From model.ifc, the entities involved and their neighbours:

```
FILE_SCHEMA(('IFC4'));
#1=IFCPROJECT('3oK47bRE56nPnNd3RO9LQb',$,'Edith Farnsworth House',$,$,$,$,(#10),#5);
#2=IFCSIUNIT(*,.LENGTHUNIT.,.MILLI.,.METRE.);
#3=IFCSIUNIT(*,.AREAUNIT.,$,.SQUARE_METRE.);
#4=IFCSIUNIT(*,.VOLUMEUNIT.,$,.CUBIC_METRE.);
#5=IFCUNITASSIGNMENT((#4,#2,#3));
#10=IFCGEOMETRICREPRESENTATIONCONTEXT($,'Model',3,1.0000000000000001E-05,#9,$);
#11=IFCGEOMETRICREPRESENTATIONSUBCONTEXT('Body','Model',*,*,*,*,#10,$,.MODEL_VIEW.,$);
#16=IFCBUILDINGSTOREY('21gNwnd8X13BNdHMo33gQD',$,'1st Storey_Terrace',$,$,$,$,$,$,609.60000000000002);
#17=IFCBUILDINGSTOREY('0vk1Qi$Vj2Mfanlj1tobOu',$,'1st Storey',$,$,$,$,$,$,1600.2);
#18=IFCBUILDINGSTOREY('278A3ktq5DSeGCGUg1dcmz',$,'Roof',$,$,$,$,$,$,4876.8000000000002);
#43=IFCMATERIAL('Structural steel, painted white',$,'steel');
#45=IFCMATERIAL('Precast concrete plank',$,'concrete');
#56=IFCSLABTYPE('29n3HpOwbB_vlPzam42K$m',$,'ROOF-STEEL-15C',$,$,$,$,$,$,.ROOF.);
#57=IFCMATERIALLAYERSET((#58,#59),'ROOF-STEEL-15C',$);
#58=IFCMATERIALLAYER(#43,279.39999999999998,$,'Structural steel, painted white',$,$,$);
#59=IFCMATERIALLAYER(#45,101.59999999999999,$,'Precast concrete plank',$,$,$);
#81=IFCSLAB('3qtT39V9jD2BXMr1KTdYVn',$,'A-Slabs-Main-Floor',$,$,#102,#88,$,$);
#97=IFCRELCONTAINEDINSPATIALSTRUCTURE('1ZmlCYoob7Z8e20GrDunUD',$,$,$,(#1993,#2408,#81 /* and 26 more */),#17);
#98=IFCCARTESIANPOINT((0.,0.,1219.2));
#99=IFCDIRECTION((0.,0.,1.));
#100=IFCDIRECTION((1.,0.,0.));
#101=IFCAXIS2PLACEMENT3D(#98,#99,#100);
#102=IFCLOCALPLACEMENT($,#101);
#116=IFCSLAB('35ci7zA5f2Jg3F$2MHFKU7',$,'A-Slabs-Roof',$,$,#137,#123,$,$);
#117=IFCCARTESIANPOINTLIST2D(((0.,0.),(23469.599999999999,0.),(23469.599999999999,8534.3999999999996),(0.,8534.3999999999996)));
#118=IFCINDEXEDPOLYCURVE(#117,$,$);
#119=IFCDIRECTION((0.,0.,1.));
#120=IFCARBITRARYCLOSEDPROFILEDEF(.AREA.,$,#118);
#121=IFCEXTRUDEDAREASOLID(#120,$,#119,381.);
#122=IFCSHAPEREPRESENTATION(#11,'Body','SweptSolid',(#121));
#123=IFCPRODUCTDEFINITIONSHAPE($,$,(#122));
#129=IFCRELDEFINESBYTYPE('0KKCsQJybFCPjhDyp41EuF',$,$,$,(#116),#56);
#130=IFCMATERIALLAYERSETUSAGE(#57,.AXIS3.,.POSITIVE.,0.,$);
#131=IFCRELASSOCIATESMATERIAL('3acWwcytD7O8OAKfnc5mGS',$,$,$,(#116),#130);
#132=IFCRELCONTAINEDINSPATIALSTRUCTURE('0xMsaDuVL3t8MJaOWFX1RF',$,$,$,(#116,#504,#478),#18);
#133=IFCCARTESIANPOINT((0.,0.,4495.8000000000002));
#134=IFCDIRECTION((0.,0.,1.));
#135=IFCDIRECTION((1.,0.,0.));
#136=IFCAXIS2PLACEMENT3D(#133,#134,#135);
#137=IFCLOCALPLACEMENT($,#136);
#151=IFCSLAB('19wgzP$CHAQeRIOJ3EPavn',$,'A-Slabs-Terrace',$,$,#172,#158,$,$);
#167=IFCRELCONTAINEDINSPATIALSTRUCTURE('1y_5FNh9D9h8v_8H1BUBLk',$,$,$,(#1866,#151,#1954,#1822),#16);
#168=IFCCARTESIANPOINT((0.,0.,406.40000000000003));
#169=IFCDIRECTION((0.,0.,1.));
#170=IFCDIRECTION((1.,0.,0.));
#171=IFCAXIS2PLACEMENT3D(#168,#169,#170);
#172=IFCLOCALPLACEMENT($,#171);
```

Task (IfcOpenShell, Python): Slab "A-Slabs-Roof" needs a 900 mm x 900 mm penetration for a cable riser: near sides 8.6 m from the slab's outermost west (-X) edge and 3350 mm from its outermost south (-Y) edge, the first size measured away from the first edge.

```python
import numpy as np
import ifcopenshell
import ifcopenshell.api.feature
import ifcopenshell.api.geometry
import ifcopenshell.api.root
import ifcopenshell.geom
import ifcopenshell.util.placement
import ifcopenshell.util.representation
import ifcopenshell.util.shape
import ifcopenshell.util.unit

model = ifcopenshell.open("model.ifc")
unit_scale = ifcopenshell.util.unit.calculate_unit_scale(model)
settings = ifcopenshell.geom.settings()


def volume(element):
    """Net volume in cubic metres, openings subtracted."""
    shape = ifcopenshell.geom.create_shape(settings, element)
    return ifcopenshell.util.shape.get_volume(shape.geometry)


slab = model.by_guid("35ci7zA5f2Jg3F$2MHFKU7")
before = volume(slab)

# Extent in the slab's own axes, in metres. The edges named are its -X and -Y sides.
slab_shape = ifcopenshell.geom.create_shape(settings, slab)
vertices = ifcopenshell.util.shape.get_vertices(slab_shape.geometry)
x_min, y_min, bottom = vertices.min(axis=0)
top = vertices[:, 2].max()

opening = ifcopenshell.api.root.create_entity(model, ifc_class="IfcOpeningElement", name="Cable riser opening", predefined_type="OPENING")
context = ifcopenshell.util.representation.get_context(model, "Model", "Body", "MODEL_VIEW")
width, depth = 0.9, 0.9
outline = [(0.0, 0.0), (width, 0.0), (width, depth), (0.0, depth), (0.0, 0.0)]
# Overshoot both faces by 50 mm so the cut is clean.
shape = ifcopenshell.api.geometry.add_slab_representation(
    model, context=context, depth=top - bottom + 0.1, polyline=outline
)
ifcopenshell.api.geometry.assign_representation(model, product=opening, representation=shape)

matrix = ifcopenshell.util.placement.get_local_placement(slab.ObjectPlacement)
matrix[:, 3] = matrix @ np.append(np.array([x_min + 8.6, y_min + 3.35, bottom - 0.05]) / unit_scale, 1.0)
ifcopenshell.api.geometry.edit_object_placement(model, product=opening, matrix=matrix, is_si=False)
ifcopenshell.api.feature.add_feature(model, feature=opening, element=slab)

after = volume(slab)

print(f"slab volume {before:.3f} -> {after:.3f} m3")

model.write("model_v2.ifc")
```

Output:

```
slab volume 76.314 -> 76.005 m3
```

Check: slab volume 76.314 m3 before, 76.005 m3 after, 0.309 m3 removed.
